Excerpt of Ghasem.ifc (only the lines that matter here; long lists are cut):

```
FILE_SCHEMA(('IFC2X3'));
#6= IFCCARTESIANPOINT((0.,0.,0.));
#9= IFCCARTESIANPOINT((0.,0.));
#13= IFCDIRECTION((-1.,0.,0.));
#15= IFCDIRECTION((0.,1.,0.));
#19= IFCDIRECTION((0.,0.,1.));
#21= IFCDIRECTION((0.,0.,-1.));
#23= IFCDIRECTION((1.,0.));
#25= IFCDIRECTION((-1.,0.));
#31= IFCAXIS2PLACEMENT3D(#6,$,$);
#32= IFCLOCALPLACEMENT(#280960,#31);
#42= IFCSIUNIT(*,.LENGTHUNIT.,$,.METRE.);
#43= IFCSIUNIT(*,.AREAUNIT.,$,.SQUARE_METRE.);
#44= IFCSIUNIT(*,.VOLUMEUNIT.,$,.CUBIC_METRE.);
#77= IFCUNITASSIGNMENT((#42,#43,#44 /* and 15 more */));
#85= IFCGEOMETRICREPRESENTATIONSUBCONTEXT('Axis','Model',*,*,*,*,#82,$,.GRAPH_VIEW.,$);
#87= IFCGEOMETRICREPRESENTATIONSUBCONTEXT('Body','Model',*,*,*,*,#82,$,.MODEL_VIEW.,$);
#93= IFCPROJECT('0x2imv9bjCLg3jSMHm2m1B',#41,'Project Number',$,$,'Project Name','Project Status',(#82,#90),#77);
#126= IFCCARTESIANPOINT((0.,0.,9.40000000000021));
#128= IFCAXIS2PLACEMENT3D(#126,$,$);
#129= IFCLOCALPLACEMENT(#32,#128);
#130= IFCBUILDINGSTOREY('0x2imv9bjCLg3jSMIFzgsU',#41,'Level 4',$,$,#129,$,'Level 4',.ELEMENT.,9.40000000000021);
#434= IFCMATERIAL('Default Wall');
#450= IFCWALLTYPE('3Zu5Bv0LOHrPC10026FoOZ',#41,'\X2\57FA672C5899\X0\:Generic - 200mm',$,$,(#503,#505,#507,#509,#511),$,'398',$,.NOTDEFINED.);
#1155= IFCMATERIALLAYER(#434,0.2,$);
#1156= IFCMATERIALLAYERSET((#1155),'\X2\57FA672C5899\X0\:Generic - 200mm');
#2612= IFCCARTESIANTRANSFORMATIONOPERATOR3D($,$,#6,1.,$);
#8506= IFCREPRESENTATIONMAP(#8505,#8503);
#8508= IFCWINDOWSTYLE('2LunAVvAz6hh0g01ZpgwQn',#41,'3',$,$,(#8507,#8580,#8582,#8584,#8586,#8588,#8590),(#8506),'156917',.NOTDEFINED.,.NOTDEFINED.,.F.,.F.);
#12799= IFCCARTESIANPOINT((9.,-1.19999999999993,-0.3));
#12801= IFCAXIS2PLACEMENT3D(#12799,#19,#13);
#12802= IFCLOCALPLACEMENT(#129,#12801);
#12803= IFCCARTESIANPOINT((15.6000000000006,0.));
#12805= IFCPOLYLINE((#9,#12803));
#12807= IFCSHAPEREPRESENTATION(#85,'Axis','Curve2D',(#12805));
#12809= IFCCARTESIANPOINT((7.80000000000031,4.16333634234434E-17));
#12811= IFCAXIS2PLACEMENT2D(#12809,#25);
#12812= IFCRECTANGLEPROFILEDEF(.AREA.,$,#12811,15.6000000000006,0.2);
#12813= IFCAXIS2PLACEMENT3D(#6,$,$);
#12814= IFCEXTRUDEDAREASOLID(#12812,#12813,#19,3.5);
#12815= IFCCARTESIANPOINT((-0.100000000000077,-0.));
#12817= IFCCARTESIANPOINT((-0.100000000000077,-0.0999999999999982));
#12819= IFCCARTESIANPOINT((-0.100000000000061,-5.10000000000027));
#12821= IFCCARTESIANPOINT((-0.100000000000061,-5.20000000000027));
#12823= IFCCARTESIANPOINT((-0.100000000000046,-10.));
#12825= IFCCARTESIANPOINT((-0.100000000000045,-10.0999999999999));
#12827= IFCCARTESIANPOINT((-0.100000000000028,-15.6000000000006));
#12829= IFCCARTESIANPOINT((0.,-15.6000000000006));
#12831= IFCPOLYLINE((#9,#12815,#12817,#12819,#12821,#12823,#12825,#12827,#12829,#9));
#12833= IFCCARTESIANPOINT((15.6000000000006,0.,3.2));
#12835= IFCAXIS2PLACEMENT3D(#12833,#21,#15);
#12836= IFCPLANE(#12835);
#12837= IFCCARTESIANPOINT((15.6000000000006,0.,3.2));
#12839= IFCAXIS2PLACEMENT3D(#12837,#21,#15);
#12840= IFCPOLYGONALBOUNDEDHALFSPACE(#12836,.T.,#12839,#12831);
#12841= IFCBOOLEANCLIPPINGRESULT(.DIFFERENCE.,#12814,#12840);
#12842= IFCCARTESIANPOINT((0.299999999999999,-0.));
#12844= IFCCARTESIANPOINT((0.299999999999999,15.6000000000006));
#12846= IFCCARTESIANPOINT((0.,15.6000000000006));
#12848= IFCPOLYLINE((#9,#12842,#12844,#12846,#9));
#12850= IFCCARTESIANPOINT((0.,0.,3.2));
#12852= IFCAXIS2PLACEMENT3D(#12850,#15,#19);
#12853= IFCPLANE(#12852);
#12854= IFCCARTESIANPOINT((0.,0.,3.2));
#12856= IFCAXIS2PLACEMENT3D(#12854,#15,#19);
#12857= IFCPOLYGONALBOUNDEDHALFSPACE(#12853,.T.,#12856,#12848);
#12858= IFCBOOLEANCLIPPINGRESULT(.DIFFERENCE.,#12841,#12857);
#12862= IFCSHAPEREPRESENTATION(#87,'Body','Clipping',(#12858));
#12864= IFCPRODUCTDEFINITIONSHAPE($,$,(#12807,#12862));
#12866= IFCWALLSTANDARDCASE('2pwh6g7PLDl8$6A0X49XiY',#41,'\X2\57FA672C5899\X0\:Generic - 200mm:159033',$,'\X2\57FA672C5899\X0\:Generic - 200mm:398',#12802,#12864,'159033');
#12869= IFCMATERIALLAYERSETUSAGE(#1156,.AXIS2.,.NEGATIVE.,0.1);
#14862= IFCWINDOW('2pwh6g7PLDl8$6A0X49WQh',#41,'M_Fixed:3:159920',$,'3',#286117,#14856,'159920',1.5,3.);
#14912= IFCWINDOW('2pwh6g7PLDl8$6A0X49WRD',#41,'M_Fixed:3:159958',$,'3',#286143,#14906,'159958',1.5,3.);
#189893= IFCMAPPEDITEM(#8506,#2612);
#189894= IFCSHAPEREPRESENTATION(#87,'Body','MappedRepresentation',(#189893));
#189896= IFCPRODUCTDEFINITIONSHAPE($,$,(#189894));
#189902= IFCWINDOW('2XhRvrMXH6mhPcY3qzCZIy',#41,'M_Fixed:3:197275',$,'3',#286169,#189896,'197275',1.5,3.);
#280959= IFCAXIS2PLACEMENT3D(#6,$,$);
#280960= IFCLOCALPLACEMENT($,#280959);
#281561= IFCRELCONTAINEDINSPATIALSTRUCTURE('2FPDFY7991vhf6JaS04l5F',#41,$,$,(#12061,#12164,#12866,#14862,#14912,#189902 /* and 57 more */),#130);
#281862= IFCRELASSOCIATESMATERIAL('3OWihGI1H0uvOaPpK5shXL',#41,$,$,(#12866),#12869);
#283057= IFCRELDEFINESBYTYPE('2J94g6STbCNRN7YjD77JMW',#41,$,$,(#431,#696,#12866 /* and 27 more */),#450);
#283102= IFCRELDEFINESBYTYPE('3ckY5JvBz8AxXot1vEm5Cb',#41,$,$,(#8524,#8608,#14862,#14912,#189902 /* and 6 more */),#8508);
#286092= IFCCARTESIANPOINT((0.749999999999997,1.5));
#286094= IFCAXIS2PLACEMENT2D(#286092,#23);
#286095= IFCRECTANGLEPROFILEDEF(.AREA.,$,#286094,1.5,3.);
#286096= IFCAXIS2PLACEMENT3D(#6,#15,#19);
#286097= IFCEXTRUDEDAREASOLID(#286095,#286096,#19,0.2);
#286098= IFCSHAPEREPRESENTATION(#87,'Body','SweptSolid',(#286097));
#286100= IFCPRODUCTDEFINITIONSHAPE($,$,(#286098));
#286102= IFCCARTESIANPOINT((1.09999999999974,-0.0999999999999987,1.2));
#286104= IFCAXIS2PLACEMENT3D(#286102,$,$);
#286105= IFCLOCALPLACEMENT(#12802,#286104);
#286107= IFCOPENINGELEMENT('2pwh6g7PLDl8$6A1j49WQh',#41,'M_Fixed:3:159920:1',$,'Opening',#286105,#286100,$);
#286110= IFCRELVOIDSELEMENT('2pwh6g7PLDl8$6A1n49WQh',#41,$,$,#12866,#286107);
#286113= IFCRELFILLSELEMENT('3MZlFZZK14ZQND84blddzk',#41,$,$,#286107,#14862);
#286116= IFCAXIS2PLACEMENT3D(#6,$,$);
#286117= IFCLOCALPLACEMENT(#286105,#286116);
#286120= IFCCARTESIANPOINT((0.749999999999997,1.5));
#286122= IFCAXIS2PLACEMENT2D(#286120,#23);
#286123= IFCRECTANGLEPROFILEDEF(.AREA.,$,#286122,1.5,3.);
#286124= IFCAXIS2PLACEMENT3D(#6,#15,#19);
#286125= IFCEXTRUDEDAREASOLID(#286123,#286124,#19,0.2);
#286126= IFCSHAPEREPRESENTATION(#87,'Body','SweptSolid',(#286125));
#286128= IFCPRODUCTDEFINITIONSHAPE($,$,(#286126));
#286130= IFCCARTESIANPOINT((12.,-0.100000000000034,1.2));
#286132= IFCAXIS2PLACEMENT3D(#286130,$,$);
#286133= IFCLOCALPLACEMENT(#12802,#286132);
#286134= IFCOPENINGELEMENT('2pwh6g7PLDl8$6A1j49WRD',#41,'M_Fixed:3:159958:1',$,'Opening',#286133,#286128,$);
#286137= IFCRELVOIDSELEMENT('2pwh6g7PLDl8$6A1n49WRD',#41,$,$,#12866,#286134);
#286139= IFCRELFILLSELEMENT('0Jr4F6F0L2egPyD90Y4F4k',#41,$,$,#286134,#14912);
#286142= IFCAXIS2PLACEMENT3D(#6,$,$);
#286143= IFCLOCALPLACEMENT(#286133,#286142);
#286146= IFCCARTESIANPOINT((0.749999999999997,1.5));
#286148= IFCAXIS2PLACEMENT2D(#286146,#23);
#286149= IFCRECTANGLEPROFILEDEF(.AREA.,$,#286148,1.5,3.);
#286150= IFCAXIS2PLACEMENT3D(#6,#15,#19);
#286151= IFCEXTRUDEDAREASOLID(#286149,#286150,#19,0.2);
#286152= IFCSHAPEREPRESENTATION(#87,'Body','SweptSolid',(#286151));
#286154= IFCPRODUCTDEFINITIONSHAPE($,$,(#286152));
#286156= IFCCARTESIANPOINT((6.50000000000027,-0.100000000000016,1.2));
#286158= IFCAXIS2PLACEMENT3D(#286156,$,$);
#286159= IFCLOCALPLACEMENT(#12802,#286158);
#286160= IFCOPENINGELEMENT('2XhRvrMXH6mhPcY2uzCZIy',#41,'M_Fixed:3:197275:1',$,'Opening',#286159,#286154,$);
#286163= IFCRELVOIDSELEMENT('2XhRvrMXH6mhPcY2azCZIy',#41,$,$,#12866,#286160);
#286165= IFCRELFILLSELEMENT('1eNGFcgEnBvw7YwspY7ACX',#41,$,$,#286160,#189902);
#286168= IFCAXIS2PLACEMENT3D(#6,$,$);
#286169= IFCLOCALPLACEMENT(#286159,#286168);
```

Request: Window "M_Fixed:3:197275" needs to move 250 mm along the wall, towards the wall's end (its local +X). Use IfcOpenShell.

```python
import ifcopenshell
import ifcopenshell.api.geometry
import ifcopenshell.util.placement

model = ifcopenshell.open("Ghasem.ifc")

window = model.by_guid("2XhRvrMXH6mhPcY3qzCZIy")
opening = window.FillsVoids[0].RelatingOpeningElement
wall = opening.VoidsElements[0].RelatingBuildingElement

wall_matrix = ifcopenshell.util.placement.get_local_placement(wall.ObjectPlacement)
shift = wall_matrix[:3, 0] * 0.25
before = ifcopenshell.util.placement.get_local_placement(window.ObjectPlacement)[:3, 3].copy()

# The window is placed relative to its opening, so it follows when the opening moves.
matrix = ifcopenshell.util.placement.get_local_placement(opening.ObjectPlacement)
matrix[:3, 3] += shift
ifcopenshell.api.geometry.edit_object_placement(
    model, product=opening, matrix=matrix, is_si=False, should_transform_children=True
)

after = ifcopenshell.util.placement.get_local_placement(window.ObjectPlacement)[:3, 3]
print("window moved by", (after - before).round(3) + 0.0)

model.write("Ghasem_updated.ifc")
```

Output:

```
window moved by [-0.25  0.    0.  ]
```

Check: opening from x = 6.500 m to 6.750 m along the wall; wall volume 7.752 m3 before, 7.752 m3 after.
